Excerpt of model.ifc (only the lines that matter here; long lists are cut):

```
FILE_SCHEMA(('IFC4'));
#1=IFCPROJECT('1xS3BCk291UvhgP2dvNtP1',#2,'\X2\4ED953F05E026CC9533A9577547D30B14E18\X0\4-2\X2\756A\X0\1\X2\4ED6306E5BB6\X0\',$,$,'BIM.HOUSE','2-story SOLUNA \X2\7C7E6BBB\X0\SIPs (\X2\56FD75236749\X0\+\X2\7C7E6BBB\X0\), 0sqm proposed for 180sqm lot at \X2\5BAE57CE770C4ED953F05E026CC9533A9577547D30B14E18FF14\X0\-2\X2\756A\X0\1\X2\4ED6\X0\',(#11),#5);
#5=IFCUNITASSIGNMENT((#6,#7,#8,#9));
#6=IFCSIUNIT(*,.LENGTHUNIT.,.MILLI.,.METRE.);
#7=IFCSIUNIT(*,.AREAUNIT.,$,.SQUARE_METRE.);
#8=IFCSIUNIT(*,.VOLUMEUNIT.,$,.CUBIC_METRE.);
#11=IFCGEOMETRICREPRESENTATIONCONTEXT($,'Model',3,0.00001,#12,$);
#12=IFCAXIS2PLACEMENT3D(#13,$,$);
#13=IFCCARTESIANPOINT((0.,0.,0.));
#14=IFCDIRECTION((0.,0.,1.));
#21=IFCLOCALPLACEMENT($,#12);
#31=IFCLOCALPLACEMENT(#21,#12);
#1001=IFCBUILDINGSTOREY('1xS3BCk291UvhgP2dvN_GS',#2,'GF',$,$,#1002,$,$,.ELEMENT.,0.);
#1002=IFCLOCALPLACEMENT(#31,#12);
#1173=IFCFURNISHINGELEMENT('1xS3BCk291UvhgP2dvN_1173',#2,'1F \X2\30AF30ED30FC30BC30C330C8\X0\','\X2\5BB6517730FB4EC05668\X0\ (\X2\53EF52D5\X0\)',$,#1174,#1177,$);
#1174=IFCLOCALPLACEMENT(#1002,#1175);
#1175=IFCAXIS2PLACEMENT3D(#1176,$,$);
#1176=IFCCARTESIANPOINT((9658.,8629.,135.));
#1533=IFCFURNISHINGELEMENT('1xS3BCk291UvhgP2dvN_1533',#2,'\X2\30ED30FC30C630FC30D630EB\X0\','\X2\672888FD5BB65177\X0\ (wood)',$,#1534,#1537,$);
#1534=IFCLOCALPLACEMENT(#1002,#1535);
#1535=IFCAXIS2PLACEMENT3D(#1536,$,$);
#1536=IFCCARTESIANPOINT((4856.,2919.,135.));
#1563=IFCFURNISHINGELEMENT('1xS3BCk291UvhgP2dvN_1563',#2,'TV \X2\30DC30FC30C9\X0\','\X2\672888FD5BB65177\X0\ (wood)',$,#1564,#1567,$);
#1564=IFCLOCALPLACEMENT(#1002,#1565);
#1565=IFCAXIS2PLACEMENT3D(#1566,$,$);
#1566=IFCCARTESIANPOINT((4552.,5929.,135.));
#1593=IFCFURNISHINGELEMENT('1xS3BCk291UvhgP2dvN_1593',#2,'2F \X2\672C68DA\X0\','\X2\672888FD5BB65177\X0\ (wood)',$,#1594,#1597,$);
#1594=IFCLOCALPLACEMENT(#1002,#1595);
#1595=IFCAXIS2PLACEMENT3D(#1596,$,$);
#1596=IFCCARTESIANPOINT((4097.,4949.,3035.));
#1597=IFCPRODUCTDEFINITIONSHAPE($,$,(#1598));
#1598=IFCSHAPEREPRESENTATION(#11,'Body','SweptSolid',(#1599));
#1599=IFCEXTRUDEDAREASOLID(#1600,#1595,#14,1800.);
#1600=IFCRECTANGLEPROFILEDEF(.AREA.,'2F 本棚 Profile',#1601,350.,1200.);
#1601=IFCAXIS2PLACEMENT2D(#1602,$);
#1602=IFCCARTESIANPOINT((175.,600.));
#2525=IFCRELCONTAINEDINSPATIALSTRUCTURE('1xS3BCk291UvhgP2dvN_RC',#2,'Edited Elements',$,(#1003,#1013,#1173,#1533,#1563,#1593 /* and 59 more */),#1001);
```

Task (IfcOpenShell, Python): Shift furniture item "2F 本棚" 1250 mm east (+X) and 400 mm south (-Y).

```python
import ifcopenshell
import ifcopenshell.api.geometry
import ifcopenshell.util.placement
import ifcopenshell.util.unit

model = ifcopenshell.open("model.ifc")
unit_scale = ifcopenshell.util.unit.calculate_unit_scale(model)

item = model.by_guid("1xS3BCk291UvhgP2dvN_1593")
matrix = ifcopenshell.util.placement.get_local_placement(item.ObjectPlacement)
matrix[0, 3] += 1.25 / unit_scale
matrix[1, 3] -= 0.4 / unit_scale
ifcopenshell.api.geometry.edit_object_placement(model, product=item, matrix=matrix, is_si=False)

print(ifcopenshell.util.placement.get_local_placement(item.ObjectPlacement).round(3) + 0.0)

model.write("model_edited.ifc")
```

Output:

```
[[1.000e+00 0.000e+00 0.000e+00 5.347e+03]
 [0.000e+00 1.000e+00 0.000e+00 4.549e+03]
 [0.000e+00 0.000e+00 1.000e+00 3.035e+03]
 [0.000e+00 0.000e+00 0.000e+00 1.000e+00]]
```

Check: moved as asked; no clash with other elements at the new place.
